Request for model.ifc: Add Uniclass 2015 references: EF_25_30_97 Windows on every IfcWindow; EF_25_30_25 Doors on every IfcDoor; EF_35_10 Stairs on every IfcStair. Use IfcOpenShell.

First a look at what the model holds.

```python
import ifcopenshell

model = ifcopenshell.open("model.ifc")
print(model.schema)
print("classifications:", [c.Name for c in model.by_type("IfcClassification")])
for ifc_class in ("IfcDoor", "IfcRoof", "IfcStair", "IfcWall", "IfcWindow"):
    print(ifc_class, len(model.by_type(ifc_class)))
```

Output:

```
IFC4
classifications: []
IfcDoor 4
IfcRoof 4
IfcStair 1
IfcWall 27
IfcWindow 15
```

```python
import ifcopenshell
import ifcopenshell.api.classification

model = ifcopenshell.open("model.ifc")

system = ifcopenshell.api.classification.add_classification(model, classification="Uniclass 2015")

codes = {
    "IfcWindow": ("EF_25_30_97", "Windows"),
    "IfcDoor": ("EF_25_30_25", "Doors"),
    "IfcStair": ("EF_35_10", "Stairs"),
}
for ifc_class, (code, name) in codes.items():
    products = model.by_type(ifc_class)
    ifcopenshell.api.classification.add_reference(
        model, products=products, classification=system, identification=code, name=name
    )
    print(code, len(products))

model.write("model_rev.ifc")
```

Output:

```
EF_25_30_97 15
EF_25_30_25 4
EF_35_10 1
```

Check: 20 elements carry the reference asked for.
